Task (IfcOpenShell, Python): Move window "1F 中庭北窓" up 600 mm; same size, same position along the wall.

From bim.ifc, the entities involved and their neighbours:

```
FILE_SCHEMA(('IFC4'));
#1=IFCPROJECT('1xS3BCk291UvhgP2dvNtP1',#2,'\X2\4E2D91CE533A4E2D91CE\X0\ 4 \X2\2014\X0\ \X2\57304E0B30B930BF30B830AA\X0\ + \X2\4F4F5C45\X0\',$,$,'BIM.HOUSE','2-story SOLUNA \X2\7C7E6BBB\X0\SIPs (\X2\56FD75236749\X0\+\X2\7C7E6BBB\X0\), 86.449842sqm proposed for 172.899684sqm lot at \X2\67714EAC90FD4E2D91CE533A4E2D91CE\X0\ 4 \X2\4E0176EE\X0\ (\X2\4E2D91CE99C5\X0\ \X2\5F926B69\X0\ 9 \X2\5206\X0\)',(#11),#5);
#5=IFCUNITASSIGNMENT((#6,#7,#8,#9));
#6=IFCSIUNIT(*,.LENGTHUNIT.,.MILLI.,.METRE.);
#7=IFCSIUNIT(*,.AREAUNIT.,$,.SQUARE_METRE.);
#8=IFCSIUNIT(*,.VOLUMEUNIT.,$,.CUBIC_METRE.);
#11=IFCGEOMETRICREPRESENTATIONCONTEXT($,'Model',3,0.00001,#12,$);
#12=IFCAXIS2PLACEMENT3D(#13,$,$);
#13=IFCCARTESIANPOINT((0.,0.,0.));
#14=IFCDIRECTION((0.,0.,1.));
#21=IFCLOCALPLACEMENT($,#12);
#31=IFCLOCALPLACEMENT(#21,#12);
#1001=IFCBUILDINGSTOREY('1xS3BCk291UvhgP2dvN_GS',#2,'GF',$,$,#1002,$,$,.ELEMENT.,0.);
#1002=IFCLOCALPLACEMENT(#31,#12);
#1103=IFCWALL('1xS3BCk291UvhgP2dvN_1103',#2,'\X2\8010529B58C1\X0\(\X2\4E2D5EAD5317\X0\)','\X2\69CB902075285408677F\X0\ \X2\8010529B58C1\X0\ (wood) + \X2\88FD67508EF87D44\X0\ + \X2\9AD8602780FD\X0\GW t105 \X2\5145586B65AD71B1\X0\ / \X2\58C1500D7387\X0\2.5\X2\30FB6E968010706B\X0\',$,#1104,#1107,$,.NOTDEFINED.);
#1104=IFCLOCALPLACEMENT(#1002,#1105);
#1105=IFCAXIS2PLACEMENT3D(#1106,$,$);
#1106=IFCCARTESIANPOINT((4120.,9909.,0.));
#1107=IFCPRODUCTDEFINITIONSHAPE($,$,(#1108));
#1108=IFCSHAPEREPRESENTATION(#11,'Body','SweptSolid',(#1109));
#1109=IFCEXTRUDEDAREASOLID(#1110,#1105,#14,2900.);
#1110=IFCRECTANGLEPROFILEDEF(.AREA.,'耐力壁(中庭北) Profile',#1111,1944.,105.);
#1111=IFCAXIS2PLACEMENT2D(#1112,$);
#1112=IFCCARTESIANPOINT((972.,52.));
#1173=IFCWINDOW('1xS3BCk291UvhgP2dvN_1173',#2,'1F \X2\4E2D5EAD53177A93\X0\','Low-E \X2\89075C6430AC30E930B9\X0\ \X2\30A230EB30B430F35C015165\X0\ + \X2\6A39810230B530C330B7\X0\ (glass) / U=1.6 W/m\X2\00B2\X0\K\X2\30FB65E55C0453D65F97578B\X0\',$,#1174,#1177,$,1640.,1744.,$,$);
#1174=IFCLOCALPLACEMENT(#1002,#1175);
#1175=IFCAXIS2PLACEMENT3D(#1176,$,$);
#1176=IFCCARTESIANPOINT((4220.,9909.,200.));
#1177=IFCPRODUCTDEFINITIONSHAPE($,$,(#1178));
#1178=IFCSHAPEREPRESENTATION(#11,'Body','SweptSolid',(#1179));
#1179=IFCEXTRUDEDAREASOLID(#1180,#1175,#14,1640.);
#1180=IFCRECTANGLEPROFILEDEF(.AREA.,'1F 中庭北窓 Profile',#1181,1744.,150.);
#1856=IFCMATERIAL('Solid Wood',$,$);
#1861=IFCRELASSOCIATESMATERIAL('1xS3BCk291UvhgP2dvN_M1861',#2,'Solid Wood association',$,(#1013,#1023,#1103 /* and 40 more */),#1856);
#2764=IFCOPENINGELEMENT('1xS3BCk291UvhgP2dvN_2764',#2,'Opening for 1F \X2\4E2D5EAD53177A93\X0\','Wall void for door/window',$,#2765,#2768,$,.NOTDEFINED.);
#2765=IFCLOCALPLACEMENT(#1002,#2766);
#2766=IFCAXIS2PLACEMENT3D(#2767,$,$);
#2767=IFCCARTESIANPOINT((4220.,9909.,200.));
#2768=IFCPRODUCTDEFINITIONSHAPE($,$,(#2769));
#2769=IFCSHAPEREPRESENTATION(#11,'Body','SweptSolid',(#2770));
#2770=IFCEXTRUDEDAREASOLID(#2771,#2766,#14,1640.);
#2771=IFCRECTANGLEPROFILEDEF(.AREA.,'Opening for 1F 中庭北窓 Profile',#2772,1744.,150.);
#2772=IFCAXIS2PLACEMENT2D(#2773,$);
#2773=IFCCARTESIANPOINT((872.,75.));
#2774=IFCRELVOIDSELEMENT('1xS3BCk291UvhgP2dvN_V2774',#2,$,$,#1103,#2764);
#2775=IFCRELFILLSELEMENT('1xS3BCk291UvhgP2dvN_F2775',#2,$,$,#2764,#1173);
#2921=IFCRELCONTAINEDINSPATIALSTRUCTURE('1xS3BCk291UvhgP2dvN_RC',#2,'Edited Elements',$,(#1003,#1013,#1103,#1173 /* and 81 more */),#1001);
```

```python
import numpy as np
import ifcopenshell
import ifcopenshell.api.geometry
import ifcopenshell.util.placement
import ifcopenshell.util.unit

model = ifcopenshell.open("bim.ifc")
unit_scale = ifcopenshell.util.unit.calculate_unit_scale(model)

window = model.by_id(1173)
opening = window.FillsVoids[0].RelatingOpeningElement
dz = 0.6 / unit_scale

shift = np.array([0.0, 0.0, dz])
# The window is not placed relative to its opening, so move both.
for product in (opening, window):
    matrix = ifcopenshell.util.placement.get_local_placement(product.ObjectPlacement)
    matrix[:3, 3] += shift
    ifcopenshell.api.geometry.edit_object_placement(model, product=product, matrix=matrix, is_si=False)

print(f"moved by {dz * unit_scale:+.3f} m")

model.write("bim_edited.ifc")
```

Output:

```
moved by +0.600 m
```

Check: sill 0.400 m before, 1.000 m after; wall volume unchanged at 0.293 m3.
